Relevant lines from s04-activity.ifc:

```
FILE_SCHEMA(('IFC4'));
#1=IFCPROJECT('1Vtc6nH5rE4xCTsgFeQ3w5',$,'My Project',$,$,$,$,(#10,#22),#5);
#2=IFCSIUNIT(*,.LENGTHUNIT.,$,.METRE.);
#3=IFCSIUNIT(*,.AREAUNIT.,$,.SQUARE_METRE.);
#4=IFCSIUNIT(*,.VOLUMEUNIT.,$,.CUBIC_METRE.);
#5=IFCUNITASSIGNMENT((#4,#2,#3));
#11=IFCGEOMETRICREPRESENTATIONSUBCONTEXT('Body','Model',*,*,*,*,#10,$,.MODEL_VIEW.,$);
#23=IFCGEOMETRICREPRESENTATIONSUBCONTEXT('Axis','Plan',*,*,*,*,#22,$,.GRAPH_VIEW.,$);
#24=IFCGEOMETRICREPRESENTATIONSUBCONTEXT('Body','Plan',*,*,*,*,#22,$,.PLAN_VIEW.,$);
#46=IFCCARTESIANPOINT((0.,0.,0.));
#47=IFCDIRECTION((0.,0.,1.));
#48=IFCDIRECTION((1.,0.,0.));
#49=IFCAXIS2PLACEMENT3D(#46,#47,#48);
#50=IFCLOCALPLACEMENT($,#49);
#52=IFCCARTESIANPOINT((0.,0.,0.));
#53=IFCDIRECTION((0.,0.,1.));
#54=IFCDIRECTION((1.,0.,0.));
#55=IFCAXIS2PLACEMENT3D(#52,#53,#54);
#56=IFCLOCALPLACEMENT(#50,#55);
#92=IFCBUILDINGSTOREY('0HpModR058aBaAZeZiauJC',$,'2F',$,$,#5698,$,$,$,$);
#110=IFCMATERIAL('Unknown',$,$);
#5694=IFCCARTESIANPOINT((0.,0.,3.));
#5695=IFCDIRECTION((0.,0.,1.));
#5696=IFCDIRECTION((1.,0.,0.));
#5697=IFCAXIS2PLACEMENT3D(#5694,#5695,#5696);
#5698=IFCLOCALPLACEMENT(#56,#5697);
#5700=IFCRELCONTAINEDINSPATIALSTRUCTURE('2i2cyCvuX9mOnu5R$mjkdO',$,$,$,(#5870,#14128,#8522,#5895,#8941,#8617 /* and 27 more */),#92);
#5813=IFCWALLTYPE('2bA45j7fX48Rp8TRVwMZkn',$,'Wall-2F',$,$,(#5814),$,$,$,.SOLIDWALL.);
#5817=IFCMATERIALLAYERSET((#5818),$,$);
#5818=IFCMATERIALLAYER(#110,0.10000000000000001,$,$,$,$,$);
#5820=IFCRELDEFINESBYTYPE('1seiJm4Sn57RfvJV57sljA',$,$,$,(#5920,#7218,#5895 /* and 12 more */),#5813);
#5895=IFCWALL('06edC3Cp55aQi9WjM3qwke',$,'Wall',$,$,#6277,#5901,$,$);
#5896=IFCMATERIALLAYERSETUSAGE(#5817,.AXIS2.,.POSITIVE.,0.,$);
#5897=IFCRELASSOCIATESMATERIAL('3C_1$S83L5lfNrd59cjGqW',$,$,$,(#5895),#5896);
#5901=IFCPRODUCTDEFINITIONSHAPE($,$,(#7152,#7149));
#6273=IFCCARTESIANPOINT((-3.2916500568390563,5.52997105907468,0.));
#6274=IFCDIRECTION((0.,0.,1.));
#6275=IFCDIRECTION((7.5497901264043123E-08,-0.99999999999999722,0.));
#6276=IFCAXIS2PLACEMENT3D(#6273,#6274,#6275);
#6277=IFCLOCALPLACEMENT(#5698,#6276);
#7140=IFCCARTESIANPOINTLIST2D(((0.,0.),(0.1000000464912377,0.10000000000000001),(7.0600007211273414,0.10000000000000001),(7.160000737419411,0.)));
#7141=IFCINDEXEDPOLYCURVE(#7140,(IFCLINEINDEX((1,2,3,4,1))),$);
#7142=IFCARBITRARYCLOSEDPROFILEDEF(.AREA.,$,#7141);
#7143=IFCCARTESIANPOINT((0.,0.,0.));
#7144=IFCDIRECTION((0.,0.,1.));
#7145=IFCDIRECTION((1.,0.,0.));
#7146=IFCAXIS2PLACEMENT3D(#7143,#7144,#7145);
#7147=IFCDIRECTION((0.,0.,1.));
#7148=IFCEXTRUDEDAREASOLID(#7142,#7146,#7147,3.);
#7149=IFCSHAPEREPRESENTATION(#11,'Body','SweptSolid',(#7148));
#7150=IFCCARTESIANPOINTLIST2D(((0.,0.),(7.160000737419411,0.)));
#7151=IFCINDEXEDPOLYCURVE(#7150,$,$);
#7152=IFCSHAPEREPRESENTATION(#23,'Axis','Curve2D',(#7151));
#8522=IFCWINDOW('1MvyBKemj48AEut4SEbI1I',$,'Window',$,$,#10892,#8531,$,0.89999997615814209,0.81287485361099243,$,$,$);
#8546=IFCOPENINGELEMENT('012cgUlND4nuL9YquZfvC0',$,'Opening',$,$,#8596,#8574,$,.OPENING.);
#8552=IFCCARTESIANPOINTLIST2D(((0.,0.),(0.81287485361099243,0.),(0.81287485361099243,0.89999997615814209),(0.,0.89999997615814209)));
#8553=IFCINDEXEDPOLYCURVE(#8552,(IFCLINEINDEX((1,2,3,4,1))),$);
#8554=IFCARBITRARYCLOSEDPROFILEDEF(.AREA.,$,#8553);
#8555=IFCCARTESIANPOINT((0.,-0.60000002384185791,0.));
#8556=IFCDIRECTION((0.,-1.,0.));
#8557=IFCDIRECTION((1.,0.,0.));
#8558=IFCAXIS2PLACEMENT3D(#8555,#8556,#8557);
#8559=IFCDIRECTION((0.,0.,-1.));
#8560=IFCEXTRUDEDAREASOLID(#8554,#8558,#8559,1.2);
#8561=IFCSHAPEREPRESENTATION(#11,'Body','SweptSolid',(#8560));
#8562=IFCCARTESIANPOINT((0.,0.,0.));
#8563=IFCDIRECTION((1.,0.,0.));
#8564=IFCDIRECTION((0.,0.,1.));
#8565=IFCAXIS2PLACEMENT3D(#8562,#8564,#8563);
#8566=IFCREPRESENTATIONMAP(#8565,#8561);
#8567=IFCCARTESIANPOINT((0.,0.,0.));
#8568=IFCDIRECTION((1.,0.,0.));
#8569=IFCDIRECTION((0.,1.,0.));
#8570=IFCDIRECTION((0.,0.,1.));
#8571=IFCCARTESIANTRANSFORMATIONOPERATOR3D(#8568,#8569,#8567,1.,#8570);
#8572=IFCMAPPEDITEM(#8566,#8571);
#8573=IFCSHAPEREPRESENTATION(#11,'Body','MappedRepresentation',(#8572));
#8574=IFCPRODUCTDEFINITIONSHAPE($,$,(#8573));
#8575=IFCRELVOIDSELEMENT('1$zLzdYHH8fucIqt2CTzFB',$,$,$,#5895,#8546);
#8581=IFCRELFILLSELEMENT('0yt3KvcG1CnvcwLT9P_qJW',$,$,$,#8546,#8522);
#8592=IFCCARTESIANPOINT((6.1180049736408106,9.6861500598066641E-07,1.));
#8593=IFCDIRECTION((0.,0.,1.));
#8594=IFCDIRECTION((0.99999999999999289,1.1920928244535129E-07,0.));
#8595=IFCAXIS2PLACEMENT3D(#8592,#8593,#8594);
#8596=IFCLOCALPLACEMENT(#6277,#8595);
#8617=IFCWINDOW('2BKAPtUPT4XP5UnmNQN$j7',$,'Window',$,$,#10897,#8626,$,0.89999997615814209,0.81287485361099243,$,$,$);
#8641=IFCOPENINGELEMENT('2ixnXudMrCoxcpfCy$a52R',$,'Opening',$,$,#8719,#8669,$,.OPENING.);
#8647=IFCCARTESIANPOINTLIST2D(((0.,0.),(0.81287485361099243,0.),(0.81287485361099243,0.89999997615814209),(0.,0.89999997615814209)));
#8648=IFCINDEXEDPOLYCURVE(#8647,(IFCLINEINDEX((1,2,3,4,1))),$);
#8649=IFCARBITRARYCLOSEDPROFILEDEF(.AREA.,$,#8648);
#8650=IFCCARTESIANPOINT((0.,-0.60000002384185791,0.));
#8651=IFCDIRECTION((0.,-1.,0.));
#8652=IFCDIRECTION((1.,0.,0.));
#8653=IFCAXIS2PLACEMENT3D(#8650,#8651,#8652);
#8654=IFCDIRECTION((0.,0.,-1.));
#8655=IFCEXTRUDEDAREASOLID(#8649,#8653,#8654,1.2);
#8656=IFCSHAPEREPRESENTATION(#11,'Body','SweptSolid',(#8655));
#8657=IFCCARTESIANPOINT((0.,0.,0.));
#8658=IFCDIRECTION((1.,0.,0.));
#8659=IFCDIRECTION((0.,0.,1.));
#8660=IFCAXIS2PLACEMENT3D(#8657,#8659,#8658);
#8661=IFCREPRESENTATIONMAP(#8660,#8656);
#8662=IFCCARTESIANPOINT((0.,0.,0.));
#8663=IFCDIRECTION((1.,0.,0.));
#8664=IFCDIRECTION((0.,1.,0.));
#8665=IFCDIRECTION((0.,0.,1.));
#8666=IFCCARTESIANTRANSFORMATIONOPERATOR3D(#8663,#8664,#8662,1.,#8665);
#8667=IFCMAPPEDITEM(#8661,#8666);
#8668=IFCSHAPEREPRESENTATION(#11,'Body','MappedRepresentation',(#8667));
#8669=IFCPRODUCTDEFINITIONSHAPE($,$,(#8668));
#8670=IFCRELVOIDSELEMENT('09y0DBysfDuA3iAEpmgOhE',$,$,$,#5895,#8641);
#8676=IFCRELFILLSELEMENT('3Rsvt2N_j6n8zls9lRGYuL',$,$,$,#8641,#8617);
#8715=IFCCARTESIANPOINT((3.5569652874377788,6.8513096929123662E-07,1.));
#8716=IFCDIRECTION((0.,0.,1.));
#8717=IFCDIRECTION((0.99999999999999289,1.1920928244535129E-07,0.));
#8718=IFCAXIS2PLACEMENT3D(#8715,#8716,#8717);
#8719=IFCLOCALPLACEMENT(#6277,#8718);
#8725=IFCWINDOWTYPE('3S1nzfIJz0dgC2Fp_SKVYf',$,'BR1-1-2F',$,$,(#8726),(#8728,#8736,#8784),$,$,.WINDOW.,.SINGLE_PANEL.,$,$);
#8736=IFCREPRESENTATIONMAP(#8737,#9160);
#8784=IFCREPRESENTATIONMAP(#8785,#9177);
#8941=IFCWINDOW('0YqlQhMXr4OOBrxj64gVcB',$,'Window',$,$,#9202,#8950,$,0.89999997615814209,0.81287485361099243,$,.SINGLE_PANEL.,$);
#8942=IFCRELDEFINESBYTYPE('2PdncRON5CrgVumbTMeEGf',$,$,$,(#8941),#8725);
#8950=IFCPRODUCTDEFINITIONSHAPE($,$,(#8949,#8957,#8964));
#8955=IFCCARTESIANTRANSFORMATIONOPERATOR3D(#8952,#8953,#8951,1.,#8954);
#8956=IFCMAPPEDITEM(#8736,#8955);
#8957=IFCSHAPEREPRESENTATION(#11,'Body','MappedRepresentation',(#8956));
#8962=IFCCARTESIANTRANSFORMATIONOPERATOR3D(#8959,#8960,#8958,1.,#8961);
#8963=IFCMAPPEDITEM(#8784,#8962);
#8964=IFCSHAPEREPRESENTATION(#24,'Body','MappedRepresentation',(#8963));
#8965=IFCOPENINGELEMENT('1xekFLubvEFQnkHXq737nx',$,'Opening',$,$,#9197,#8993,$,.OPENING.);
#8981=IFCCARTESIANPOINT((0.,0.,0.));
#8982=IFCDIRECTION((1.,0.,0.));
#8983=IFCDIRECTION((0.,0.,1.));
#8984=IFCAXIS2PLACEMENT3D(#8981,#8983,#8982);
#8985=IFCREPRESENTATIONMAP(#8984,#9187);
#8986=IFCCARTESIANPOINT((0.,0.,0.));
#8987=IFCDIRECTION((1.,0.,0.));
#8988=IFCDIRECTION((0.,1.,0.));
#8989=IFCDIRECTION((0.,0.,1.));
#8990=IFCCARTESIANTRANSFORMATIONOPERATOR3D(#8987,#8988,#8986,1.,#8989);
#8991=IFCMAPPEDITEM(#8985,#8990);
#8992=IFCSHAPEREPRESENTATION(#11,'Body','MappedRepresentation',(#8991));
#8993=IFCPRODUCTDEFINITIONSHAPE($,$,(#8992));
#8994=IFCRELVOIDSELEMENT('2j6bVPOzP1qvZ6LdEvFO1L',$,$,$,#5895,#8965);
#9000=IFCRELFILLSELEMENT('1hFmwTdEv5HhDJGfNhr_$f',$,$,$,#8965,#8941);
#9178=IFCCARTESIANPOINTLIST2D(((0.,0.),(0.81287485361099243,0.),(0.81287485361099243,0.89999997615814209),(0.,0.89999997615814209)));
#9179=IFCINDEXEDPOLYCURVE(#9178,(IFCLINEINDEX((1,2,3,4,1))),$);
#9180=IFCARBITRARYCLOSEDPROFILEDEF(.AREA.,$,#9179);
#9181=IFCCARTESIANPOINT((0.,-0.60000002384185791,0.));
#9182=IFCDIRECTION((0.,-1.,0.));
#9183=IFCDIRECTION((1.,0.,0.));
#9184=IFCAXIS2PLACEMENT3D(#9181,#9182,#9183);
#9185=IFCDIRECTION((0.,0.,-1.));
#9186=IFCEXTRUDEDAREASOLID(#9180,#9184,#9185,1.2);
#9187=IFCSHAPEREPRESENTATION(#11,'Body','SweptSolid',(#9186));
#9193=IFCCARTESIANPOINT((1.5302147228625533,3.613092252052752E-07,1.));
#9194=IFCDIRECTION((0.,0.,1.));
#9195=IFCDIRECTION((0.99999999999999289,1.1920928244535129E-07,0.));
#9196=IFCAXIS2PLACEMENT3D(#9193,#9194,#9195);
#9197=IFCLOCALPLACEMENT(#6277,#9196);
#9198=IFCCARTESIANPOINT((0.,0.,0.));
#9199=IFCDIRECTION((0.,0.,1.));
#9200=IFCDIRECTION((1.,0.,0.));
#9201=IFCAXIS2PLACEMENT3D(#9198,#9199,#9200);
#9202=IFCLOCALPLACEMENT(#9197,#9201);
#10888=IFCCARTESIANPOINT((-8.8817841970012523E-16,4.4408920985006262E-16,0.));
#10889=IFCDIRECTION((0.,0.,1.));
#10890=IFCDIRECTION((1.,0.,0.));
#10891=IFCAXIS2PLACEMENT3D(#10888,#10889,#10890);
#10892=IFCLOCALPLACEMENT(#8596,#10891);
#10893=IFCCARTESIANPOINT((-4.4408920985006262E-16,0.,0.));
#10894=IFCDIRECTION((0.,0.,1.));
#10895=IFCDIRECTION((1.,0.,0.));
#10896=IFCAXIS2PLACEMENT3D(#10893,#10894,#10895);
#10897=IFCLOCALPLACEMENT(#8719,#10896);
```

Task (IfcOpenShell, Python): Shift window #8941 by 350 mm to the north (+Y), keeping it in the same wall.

```python
import ifcopenshell
import ifcopenshell.api.geometry
import ifcopenshell.util.placement
import ifcopenshell.util.unit

model = ifcopenshell.open("s04-activity.ifc")
unit_scale = ifcopenshell.util.unit.calculate_unit_scale(model)

window = model.by_guid("0YqlQhMXr4OOBrxj64gVcB")
opening = window.FillsVoids[0].RelatingOpeningElement
wall = opening.VoidsElements[0].RelatingBuildingElement

wall_matrix = ifcopenshell.util.placement.get_local_placement(wall.ObjectPlacement)
shift = wall_matrix[:3, 0] * -0.35 / unit_scale
before = ifcopenshell.util.placement.get_local_placement(window.ObjectPlacement)[:3, 3].copy()

# The window is placed relative to its opening, so it follows when the opening moves.
matrix = ifcopenshell.util.placement.get_local_placement(opening.ObjectPlacement)
matrix[:3, 3] += shift
ifcopenshell.api.geometry.edit_object_placement(
    model, product=opening, matrix=matrix, is_si=False, should_transform_children=True
)

after = ifcopenshell.util.placement.get_local_placement(window.ObjectPlacement)[:3, 3]
print("window moved by", (after - before).round(3) + 0.0)

model.write("s04-activity_v2.ifc")
```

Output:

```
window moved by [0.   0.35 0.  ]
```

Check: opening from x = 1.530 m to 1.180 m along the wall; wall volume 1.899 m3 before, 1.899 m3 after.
